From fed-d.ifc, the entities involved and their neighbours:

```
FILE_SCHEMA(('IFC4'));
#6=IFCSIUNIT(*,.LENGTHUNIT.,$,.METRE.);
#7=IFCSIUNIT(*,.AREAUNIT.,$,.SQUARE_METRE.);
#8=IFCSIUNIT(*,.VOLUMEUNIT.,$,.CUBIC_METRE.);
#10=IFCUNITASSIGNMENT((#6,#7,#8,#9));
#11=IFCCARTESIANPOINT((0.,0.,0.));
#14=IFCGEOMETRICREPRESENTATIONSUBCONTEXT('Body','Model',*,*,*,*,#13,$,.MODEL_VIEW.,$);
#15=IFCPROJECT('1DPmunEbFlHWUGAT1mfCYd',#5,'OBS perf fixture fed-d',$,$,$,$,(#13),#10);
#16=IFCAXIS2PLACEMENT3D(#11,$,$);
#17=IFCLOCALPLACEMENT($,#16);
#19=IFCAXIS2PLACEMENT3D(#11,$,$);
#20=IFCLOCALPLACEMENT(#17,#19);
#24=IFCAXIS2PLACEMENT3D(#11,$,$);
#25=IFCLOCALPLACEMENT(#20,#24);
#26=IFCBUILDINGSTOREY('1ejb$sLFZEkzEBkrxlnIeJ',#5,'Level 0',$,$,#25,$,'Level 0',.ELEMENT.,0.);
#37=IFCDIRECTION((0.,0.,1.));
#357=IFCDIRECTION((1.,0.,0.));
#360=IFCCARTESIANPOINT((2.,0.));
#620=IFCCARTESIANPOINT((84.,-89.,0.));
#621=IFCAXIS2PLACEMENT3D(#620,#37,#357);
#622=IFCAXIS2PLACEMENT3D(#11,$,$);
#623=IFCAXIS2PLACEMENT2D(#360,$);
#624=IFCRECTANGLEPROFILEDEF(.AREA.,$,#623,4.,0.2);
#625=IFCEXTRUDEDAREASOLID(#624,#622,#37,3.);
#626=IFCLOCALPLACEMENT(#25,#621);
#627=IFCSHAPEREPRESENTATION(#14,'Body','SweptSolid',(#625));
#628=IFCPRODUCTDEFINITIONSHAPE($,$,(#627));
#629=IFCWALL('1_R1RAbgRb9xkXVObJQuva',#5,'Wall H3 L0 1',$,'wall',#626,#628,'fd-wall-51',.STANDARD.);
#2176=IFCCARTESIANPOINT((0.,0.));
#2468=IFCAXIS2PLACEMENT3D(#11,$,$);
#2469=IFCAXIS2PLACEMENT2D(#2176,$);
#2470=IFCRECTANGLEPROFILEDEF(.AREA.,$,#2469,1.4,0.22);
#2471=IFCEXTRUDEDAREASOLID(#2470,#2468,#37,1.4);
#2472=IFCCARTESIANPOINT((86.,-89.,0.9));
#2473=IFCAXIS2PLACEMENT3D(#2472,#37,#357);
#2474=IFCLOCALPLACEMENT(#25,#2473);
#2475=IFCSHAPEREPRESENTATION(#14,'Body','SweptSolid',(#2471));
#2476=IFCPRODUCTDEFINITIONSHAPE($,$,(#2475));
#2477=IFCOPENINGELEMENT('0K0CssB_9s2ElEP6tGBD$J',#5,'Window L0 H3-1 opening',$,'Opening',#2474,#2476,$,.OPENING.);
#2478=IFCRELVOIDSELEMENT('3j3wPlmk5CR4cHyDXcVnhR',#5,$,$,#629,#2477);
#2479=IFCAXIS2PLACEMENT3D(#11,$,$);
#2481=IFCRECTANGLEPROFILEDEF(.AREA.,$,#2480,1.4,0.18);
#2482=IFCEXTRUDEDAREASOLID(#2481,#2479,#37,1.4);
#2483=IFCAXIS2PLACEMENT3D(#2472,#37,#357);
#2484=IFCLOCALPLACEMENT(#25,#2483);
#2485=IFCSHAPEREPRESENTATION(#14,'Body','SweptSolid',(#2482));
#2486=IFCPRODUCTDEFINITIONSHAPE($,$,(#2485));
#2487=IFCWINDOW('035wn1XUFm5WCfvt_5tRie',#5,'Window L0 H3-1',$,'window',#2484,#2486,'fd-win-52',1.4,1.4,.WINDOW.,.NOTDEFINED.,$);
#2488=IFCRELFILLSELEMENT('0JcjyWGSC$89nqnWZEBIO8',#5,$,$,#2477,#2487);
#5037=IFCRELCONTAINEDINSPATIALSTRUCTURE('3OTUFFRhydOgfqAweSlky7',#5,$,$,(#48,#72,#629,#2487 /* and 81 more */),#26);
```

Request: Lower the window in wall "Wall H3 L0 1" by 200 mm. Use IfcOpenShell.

```python
import numpy as np
import ifcopenshell
import ifcopenshell.api.geometry
import ifcopenshell.util.placement
import ifcopenshell.util.unit

model = ifcopenshell.open("fed-d.ifc")
unit_scale = ifcopenshell.util.unit.calculate_unit_scale(model)

window = model.by_id(2487)
opening = window.FillsVoids[0].RelatingOpeningElement
dz = -0.2 / unit_scale

shift = np.array([0.0, 0.0, dz])
# The window is not placed relative to its opening, so move both.
for product in (opening, window):
    matrix = ifcopenshell.util.placement.get_local_placement(product.ObjectPlacement)
    matrix[:3, 3] += shift
    ifcopenshell.api.geometry.edit_object_placement(model, product=product, matrix=matrix, is_si=False)

print(f"moved by {dz * unit_scale:+.3f} m")

model.write("fed-d_edited.ifc")
```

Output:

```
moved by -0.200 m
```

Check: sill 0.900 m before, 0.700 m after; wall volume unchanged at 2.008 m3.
